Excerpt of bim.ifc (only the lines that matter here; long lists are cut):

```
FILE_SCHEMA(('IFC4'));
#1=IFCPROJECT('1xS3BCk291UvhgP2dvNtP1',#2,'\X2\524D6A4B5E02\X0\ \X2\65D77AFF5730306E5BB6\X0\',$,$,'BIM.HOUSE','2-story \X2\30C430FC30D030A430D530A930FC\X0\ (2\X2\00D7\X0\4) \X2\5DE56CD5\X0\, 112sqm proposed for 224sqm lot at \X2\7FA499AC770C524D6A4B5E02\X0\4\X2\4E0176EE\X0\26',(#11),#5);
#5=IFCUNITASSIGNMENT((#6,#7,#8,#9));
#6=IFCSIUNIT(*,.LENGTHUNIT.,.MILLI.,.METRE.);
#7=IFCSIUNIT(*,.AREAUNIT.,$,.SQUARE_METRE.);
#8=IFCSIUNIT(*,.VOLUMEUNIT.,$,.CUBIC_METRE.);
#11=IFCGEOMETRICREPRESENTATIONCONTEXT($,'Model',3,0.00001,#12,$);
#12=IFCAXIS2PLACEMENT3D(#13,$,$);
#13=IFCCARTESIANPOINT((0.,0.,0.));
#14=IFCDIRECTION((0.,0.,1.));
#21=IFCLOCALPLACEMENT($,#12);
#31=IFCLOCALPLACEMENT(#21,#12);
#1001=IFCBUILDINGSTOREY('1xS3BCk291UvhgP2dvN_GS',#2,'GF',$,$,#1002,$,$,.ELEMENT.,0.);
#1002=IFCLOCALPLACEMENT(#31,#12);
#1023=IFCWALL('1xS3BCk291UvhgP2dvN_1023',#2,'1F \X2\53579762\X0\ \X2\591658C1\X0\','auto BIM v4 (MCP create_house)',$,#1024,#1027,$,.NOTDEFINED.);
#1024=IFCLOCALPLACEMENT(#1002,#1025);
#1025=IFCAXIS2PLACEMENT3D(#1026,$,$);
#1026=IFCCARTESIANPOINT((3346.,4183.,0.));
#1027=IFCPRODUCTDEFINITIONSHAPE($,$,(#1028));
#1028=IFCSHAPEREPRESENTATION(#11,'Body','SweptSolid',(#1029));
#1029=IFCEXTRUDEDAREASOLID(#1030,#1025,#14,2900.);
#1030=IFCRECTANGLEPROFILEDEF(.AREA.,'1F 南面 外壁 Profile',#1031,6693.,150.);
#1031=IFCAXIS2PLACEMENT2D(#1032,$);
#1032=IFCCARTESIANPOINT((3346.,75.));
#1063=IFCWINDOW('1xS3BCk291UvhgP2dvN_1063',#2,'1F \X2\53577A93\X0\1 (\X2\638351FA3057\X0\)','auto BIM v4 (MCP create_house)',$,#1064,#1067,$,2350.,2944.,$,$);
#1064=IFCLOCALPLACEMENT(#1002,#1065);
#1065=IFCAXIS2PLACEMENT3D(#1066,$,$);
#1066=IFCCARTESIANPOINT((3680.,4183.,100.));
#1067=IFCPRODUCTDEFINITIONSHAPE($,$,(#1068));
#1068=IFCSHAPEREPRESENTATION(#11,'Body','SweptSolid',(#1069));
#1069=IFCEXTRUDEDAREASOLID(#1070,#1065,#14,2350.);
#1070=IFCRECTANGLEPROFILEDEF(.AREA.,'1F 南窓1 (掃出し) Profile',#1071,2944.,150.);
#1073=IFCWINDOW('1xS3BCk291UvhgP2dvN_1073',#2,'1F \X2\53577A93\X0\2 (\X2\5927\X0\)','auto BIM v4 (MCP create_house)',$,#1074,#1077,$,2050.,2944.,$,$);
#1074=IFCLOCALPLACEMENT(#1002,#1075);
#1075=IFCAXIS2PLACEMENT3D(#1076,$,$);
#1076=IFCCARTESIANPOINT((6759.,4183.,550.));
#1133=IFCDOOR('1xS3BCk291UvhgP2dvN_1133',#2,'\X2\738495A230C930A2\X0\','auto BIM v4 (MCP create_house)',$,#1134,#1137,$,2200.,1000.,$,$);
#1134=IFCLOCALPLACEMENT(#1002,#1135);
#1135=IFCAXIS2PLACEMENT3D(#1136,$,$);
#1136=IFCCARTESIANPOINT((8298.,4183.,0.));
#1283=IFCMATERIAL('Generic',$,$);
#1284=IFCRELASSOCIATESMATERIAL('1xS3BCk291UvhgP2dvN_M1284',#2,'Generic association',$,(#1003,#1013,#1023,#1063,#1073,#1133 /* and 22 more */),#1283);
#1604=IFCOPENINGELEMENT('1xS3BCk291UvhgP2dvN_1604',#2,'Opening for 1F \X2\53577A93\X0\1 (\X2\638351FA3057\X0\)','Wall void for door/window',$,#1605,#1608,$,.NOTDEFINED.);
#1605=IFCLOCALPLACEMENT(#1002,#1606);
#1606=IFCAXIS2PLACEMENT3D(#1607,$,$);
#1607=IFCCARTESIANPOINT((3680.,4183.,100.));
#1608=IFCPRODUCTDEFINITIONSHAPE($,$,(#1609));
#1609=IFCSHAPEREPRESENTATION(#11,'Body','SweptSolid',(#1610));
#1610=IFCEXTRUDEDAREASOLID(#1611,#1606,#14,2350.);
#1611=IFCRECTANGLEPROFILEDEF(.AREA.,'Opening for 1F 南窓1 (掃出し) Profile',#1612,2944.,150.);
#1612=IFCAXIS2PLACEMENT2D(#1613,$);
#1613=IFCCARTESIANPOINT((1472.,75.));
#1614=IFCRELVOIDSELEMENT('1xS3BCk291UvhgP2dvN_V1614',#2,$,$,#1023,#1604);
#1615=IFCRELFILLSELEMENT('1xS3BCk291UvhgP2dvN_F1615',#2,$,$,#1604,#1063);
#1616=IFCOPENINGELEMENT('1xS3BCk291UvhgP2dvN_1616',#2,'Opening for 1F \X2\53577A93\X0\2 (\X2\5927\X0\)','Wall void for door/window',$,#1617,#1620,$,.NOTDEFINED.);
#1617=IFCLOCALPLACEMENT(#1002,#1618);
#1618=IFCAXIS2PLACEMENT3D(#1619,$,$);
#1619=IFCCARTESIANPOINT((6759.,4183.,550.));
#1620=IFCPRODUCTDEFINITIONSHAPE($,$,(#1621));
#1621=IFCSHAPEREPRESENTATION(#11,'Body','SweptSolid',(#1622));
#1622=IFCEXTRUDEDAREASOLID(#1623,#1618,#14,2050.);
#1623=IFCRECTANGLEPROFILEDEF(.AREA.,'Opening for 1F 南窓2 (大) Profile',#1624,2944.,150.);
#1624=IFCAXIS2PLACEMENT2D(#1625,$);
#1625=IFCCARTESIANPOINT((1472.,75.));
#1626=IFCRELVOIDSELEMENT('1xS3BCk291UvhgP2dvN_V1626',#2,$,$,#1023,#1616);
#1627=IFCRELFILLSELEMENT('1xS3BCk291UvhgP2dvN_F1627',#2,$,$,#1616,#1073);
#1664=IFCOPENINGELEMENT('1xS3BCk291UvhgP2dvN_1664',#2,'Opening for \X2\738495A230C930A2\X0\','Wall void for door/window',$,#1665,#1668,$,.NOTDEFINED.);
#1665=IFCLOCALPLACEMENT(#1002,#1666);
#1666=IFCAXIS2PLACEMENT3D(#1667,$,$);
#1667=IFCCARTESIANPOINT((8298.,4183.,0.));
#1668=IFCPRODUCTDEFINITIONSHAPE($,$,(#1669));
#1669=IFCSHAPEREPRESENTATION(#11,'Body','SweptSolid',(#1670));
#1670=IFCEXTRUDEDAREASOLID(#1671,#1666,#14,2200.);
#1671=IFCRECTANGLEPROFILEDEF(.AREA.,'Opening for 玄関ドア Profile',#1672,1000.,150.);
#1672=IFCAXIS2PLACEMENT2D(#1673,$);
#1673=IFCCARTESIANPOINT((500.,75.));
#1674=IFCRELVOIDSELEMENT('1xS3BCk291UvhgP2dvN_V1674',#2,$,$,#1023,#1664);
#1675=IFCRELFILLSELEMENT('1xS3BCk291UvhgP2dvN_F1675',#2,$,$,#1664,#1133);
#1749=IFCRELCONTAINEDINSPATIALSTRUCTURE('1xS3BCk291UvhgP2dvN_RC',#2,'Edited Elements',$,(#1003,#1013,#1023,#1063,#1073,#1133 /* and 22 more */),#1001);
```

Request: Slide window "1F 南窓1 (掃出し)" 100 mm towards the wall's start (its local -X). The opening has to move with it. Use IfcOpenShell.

```python
import ifcopenshell
import ifcopenshell.api.geometry
import ifcopenshell.util.placement
import ifcopenshell.util.unit

model = ifcopenshell.open("bim.ifc")
unit_scale = ifcopenshell.util.unit.calculate_unit_scale(model)

window = model.by_guid("1xS3BCk291UvhgP2dvN_1063")
opening = window.FillsVoids[0].RelatingOpeningElement
wall = opening.VoidsElements[0].RelatingBuildingElement

wall_matrix = ifcopenshell.util.placement.get_local_placement(wall.ObjectPlacement)
shift = wall_matrix[:3, 0] * -0.1 / unit_scale
before = ifcopenshell.util.placement.get_local_placement(window.ObjectPlacement)[:3, 3].copy()

# The window is not placed relative to its opening, so move both.
for product in (opening, window):
    matrix = ifcopenshell.util.placement.get_local_placement(product.ObjectPlacement)
    matrix[:3, 3] += shift
    ifcopenshell.api.geometry.edit_object_placement(model, product=product, matrix=matrix, is_si=False)

after = ifcopenshell.util.placement.get_local_placement(window.ObjectPlacement)[:3, 3]
print("window moved by", (after - before).round(3) + 0.0)

model.write("bim_rev.ifc")
```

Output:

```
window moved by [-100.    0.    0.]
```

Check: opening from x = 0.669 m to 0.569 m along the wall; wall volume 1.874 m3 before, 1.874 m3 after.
